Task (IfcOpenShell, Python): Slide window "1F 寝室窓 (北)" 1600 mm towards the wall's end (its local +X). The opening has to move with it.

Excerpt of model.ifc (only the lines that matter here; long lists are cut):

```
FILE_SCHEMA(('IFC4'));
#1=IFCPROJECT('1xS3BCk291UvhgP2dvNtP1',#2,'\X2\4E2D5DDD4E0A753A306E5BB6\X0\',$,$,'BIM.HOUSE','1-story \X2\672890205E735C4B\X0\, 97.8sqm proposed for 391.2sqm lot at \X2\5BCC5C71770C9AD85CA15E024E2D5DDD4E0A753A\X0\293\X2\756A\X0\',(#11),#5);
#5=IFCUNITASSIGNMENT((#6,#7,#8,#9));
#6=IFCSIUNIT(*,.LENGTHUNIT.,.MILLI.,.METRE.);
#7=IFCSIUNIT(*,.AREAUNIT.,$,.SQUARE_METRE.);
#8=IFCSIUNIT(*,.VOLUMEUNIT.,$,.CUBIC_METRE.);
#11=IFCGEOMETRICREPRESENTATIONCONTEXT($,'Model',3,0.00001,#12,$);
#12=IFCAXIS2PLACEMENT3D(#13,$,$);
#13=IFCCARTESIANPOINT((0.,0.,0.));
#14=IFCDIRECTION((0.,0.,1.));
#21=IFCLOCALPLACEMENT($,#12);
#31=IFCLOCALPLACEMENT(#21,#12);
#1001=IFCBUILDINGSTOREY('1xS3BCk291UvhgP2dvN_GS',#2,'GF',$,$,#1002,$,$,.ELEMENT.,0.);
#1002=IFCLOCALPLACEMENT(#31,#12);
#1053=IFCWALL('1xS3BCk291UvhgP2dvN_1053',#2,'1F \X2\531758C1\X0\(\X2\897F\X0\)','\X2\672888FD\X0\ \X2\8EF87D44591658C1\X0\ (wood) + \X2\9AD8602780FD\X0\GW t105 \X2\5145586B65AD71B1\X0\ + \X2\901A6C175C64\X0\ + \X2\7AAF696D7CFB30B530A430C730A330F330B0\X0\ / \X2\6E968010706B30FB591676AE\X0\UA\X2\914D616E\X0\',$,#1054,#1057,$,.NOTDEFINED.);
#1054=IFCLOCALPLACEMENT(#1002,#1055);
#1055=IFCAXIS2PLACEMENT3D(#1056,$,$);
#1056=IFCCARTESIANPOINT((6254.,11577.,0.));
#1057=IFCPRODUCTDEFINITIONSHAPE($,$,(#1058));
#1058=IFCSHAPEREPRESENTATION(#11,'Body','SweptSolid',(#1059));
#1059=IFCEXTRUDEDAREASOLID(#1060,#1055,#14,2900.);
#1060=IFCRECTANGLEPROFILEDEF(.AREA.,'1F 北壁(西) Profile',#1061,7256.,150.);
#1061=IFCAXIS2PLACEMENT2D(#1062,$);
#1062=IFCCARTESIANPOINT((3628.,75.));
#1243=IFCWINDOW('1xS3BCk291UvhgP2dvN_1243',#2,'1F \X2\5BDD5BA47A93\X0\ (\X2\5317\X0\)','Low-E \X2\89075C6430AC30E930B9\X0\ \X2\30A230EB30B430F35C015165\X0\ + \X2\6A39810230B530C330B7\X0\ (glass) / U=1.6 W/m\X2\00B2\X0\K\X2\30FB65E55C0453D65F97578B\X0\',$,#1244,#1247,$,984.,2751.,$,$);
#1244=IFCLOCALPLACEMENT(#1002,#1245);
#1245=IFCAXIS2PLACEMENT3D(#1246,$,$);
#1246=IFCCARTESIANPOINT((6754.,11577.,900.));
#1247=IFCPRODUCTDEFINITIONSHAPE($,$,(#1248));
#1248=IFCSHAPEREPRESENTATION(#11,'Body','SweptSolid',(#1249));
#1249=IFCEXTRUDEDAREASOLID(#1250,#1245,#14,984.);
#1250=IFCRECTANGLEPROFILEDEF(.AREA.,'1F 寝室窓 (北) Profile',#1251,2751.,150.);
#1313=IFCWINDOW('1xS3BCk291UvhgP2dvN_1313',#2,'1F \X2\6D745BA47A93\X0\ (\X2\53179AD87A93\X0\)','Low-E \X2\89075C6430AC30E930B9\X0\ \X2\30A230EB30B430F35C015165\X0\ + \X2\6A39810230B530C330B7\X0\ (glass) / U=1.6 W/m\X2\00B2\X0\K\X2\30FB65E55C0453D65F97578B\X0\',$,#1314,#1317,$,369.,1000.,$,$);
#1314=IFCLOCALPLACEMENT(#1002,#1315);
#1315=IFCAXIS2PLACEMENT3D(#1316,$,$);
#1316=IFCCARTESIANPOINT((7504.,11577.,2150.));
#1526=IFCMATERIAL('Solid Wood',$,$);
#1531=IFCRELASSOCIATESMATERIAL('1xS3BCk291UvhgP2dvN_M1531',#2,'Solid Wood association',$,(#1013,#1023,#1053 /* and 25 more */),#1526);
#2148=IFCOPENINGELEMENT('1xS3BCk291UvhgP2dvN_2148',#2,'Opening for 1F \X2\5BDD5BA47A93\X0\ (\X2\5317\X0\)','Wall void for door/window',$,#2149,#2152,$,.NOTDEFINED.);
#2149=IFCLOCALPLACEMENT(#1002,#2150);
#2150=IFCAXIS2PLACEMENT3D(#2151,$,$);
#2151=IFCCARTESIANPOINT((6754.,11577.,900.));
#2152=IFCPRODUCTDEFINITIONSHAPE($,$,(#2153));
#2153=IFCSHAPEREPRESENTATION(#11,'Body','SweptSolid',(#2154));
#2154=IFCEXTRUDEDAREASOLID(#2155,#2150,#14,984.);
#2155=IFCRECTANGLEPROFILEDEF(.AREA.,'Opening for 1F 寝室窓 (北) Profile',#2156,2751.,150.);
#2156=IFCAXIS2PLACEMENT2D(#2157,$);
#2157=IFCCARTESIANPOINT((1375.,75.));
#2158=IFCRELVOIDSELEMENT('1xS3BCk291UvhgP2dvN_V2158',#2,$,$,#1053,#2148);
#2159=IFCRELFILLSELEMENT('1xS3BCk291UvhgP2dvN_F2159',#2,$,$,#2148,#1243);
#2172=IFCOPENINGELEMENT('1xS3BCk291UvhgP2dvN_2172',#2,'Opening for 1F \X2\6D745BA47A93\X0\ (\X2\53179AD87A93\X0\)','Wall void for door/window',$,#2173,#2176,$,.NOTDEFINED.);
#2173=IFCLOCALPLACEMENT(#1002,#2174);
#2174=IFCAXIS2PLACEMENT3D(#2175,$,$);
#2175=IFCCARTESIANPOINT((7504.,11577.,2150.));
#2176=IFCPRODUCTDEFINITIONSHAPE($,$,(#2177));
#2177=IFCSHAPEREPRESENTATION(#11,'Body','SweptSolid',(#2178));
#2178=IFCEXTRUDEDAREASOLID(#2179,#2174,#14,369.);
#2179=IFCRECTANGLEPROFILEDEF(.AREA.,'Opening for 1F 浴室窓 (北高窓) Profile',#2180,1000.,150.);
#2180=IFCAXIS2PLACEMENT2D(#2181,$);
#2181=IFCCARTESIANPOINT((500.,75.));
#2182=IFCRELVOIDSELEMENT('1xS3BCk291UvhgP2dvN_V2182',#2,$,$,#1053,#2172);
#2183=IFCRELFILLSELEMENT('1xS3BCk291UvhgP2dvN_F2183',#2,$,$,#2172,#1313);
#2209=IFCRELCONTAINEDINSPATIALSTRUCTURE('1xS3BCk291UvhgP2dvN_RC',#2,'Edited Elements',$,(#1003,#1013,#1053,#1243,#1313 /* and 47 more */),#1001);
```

```python
import ifcopenshell
import ifcopenshell.api.geometry
import ifcopenshell.util.placement

model = ifcopenshell.open("model.ifc")

window = model.by_guid("1xS3BCk291UvhgP2dvN_1243")
opening = window.FillsVoids[0].RelatingOpeningElement
wall = opening.VoidsElements[0].RelatingBuildingElement

wall_matrix = ifcopenshell.util.placement.get_local_placement(wall.ObjectPlacement)
shift = wall_matrix[:3, 0] * 1600.0
before = ifcopenshell.util.placement.get_local_placement(window.ObjectPlacement)[:3, 3].copy()

# The window is not placed relative to its opening, so move both.
for product in (opening, window):
    matrix = ifcopenshell.util.placement.get_local_placement(product.ObjectPlacement)
    matrix[:3, 3] += shift
    ifcopenshell.api.geometry.edit_object_placement(model, product=product, matrix=matrix, is_si=False)

after = ifcopenshell.util.placement.get_local_placement(window.ObjectPlacement)[:3, 3]
print("window moved by", (after - before).round(3) + 0.0)

model.write("model_updated.ifc")
```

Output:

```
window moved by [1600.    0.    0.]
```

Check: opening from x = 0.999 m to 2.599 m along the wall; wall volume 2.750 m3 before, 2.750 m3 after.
